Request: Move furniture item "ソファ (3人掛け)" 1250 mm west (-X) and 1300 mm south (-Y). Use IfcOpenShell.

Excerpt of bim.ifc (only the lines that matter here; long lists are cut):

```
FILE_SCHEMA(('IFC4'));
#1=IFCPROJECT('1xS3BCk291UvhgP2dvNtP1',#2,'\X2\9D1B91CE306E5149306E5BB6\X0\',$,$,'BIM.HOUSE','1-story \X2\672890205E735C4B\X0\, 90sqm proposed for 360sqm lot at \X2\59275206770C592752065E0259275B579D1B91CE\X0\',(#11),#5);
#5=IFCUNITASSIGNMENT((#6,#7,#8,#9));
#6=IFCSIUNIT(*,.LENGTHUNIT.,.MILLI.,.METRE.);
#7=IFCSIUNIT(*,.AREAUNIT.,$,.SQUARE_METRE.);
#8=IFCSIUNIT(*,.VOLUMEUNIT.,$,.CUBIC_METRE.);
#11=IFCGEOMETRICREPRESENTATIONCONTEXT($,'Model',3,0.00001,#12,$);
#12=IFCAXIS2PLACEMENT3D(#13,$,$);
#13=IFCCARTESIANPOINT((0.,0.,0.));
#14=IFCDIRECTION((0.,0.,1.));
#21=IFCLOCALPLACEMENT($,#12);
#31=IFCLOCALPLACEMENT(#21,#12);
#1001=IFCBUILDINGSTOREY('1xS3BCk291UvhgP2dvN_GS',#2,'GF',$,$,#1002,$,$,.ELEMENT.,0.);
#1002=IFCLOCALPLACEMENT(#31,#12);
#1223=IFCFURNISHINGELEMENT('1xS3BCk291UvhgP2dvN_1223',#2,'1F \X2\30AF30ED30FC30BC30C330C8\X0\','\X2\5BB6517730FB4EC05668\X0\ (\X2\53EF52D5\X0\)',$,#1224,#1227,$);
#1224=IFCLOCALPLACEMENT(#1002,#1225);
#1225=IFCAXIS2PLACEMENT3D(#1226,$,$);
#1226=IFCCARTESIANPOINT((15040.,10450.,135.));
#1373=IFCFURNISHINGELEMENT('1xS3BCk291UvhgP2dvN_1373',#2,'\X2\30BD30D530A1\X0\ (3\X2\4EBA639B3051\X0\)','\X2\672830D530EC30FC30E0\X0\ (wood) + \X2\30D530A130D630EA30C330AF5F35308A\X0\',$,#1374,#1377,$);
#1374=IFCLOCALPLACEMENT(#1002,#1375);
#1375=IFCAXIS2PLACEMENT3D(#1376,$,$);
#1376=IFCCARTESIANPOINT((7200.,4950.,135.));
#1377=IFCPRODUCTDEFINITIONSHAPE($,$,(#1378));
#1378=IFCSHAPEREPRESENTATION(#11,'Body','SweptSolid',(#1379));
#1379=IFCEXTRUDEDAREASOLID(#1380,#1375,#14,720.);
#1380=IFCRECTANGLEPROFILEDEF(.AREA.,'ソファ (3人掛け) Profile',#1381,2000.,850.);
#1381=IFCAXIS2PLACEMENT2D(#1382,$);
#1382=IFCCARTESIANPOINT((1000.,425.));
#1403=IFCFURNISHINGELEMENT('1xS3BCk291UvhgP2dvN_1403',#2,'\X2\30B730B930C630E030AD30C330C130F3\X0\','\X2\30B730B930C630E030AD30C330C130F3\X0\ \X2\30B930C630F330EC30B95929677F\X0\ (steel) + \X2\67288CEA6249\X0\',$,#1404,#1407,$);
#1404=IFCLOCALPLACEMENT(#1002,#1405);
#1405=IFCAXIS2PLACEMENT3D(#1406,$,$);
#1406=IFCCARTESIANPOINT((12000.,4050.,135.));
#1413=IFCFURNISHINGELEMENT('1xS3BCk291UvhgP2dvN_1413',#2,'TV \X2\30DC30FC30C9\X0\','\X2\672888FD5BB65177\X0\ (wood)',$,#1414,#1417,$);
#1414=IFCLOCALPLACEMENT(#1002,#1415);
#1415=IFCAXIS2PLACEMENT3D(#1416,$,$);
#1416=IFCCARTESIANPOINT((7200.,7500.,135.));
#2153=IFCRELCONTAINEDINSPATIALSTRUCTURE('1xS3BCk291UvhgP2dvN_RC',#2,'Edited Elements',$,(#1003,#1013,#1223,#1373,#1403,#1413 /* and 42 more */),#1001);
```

```python
import ifcopenshell
import ifcopenshell.api.geometry
import ifcopenshell.util.placement

model = ifcopenshell.open("bim.ifc")

item = model.by_guid("1xS3BCk291UvhgP2dvN_1373")
matrix = ifcopenshell.util.placement.get_local_placement(item.ObjectPlacement)
matrix[0, 3] -= 1250.0
matrix[1, 3] -= 1300.0
ifcopenshell.api.geometry.edit_object_placement(model, product=item, matrix=matrix, is_si=False)

print(ifcopenshell.util.placement.get_local_placement(item.ObjectPlacement).round(3) + 0.0)

model.write("bim-out.ifc")
```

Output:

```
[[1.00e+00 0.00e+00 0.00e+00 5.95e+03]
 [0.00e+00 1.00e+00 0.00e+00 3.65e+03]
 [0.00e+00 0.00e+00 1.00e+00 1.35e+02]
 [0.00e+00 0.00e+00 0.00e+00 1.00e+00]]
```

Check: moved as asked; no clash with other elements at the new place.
